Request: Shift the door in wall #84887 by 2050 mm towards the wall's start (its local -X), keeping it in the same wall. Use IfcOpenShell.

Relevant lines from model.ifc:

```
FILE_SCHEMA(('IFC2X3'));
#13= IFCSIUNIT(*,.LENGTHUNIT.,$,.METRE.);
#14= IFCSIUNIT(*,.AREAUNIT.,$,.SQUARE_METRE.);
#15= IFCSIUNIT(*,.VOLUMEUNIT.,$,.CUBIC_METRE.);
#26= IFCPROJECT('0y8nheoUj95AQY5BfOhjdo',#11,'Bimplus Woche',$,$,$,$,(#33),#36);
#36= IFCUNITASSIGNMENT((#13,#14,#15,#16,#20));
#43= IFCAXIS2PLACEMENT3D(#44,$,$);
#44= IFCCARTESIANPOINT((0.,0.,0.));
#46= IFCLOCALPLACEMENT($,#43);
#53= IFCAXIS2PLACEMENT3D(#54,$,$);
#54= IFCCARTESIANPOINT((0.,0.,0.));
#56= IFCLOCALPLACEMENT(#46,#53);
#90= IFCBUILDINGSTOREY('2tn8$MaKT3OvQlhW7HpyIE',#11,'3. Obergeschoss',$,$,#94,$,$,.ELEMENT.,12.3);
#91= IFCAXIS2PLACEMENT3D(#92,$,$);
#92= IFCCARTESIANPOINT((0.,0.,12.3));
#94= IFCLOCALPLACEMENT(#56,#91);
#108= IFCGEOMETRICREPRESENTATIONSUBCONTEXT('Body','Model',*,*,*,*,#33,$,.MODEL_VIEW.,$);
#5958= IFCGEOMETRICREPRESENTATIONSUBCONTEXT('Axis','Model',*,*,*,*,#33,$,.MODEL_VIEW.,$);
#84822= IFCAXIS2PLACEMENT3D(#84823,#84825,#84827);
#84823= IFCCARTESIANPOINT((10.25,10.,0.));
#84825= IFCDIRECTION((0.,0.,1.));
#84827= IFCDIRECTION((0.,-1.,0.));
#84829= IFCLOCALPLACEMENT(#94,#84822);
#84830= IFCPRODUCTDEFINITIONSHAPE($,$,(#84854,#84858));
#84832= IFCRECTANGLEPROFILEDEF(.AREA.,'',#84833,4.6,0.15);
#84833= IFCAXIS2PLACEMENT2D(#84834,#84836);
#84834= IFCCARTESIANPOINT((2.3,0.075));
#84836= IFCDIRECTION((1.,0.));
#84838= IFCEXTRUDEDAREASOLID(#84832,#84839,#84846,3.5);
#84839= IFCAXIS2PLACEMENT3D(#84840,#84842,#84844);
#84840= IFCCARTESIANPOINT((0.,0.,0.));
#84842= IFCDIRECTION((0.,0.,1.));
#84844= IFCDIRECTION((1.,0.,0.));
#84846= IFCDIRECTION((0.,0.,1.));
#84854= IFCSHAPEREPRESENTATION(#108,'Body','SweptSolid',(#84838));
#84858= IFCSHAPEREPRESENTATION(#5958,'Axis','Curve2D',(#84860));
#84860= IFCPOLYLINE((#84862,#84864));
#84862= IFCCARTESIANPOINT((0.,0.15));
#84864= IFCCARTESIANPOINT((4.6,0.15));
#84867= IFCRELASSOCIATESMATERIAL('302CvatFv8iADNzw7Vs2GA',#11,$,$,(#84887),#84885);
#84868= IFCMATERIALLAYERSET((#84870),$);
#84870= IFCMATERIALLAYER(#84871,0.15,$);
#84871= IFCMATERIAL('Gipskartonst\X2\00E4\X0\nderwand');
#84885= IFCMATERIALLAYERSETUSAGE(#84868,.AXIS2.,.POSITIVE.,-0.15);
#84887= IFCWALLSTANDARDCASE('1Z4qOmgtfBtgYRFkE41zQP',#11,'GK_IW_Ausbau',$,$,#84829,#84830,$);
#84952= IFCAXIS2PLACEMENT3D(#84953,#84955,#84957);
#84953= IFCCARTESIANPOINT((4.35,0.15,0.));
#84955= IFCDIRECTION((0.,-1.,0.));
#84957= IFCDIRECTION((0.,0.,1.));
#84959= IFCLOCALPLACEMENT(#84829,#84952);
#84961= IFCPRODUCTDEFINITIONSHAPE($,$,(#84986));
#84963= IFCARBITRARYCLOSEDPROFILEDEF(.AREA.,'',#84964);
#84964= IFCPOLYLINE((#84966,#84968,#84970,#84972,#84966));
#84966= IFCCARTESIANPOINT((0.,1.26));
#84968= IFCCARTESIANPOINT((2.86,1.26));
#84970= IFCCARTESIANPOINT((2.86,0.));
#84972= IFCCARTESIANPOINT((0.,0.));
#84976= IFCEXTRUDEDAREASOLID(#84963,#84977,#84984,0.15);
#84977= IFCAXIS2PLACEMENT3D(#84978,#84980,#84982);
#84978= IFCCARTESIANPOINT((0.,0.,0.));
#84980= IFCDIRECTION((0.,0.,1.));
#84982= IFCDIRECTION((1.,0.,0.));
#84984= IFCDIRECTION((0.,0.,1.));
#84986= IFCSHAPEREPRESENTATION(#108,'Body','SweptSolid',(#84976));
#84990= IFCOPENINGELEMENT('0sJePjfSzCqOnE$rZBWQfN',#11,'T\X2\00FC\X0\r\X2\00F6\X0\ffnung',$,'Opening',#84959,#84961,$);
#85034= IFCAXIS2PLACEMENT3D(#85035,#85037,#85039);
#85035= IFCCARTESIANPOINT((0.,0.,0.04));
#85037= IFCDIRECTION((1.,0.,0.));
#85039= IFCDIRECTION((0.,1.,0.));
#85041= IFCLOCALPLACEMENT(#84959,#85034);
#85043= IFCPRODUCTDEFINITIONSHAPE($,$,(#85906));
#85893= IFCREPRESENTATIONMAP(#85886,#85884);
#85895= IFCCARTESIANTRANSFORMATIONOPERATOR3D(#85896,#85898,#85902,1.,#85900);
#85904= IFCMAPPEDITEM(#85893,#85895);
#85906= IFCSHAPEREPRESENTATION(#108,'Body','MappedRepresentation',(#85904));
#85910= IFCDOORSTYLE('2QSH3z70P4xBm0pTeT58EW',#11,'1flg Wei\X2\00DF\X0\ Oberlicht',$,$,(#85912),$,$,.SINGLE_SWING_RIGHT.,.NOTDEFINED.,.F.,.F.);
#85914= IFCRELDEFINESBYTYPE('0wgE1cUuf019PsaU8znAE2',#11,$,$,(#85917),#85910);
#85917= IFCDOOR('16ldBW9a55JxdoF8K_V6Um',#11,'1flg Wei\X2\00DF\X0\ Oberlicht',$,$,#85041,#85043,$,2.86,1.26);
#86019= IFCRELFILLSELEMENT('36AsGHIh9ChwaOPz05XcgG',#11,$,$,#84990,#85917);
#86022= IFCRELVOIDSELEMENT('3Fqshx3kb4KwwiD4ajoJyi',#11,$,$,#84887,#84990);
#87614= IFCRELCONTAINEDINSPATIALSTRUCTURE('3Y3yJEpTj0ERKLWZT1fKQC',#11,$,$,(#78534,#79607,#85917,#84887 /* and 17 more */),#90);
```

```python
import ifcopenshell
import ifcopenshell.api.geometry
import ifcopenshell.util.placement

model = ifcopenshell.open("model.ifc")

door = model.by_guid("16ldBW9a55JxdoF8K_V6Um")
opening = door.FillsVoids[0].RelatingOpeningElement
wall = opening.VoidsElements[0].RelatingBuildingElement

wall_matrix = ifcopenshell.util.placement.get_local_placement(wall.ObjectPlacement)
shift = wall_matrix[:3, 0] * -2.05
before = ifcopenshell.util.placement.get_local_placement(door.ObjectPlacement)[:3, 3].copy()

# The door is placed relative to its opening, so it follows when the opening moves.
matrix = ifcopenshell.util.placement.get_local_placement(opening.ObjectPlacement)
matrix[:3, 3] += shift
ifcopenshell.api.geometry.edit_object_placement(
    model, product=opening, matrix=matrix, is_si=False, should_transform_children=True
)

after = ifcopenshell.util.placement.get_local_placement(door.ObjectPlacement)[:3, 3]
print("door moved by", (after - before).round(3) + 0.0)

model.write("model_edited.ifc")
```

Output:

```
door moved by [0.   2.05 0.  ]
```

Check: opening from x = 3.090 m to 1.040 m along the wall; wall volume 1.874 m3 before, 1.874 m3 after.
